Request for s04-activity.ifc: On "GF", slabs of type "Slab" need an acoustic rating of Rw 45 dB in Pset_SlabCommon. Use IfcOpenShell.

First a look at what the model holds.

```python
import ifcopenshell
import ifcopenshell.util.element

model = ifcopenshell.open("s04-activity.ifc")
print(model.schema)
storey = next(s for s in model.by_type("IfcBuildingStorey") if s.Name == "GF")
slabs = [e for e in ifcopenshell.util.element.get_decomposition(storey) if e.is_a("IfcSlab")]
seen = {}
for e in slabs:
    element_type = ifcopenshell.util.element.get_type(e)
    key = (element_type.Name if element_type != e and element_type else None, ifcopenshell.util.element.get_pset(e, "Pset_SlabCommon", "AcousticRating"))
    seen[key] = seen.get(key, 0) + 1
for (name, value), count in sorted(seen.items(), key=str):
    print(count, "x", name, "|", value)
```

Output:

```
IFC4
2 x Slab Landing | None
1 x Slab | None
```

```python
import ifcopenshell
import ifcopenshell.api.pset
import ifcopenshell.util.element

model = ifcopenshell.open("s04-activity.ifc")

storey = next(s for s in model.by_type("IfcBuildingStorey") if s.Name == "GF")
slabs = [e for e in ifcopenshell.util.element.get_decomposition(storey) if e.is_a("IfcSlab")]

count = 0
for e in slabs:
    element_type = ifcopenshell.util.element.get_type(e)
    if element_type in (None, e) or element_type.Name != "Slab":
        continue
    # add_pset returns the element's existing set when there is one.
    pset = ifcopenshell.api.pset.add_pset(model, product=e, name="Pset_SlabCommon")
    ifcopenshell.api.pset.edit_pset(model, pset=pset, properties={"AcousticRating": "Rw 45 dB"})
    count += 1

print(count, "slabs updated")

model.write("s04-activity_edited.ifc")
```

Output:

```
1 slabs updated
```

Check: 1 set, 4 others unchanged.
